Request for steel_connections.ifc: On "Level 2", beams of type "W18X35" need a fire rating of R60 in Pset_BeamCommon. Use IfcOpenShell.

First a look at what the model holds.

```python
import ifcopenshell
import ifcopenshell.util.element

model = ifcopenshell.open("steel_connections.ifc")
print(model.schema)
storey = next(s for s in model.by_type("IfcBuildingStorey") if s.Name == "Level 2")
beams = [e for e in ifcopenshell.util.element.get_decomposition(storey) if e.is_a("IfcBeam")]
seen = {}
for e in beams:
    element_type = ifcopenshell.util.element.get_type(e)
    key = (element_type.Name if element_type != e and element_type else None, ifcopenshell.util.element.get_pset(e, "Pset_BeamCommon", "FireRating"))
    seen[key] = seen.get(key, 0) + 1
for (name, value), count in sorted(seen.items(), key=str):
    print(count, "x", name, "|", value)
```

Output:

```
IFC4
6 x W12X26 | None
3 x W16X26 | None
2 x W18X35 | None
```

```python
import ifcopenshell
import ifcopenshell.api.pset
import ifcopenshell.util.element

model = ifcopenshell.open("steel_connections.ifc")

storey = next(s for s in model.by_type("IfcBuildingStorey") if s.Name == "Level 2")
beams = [e for e in ifcopenshell.util.element.get_decomposition(storey) if e.is_a("IfcBeam")]

count = 0
for e in beams:
    element_type = ifcopenshell.util.element.get_type(e)
    if element_type in (None, e) or element_type.Name != "W18X35":
        continue
    # add_pset returns the element's existing set when there is one.
    pset = ifcopenshell.api.pset.add_pset(model, product=e, name="Pset_BeamCommon")
    ifcopenshell.api.pset.edit_pset(model, pset=pset, properties={"FireRating": "R60"})
    count += 1

print(count, "beams updated")

model.write("steel_connections_updated.ifc")
```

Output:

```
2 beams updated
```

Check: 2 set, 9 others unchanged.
